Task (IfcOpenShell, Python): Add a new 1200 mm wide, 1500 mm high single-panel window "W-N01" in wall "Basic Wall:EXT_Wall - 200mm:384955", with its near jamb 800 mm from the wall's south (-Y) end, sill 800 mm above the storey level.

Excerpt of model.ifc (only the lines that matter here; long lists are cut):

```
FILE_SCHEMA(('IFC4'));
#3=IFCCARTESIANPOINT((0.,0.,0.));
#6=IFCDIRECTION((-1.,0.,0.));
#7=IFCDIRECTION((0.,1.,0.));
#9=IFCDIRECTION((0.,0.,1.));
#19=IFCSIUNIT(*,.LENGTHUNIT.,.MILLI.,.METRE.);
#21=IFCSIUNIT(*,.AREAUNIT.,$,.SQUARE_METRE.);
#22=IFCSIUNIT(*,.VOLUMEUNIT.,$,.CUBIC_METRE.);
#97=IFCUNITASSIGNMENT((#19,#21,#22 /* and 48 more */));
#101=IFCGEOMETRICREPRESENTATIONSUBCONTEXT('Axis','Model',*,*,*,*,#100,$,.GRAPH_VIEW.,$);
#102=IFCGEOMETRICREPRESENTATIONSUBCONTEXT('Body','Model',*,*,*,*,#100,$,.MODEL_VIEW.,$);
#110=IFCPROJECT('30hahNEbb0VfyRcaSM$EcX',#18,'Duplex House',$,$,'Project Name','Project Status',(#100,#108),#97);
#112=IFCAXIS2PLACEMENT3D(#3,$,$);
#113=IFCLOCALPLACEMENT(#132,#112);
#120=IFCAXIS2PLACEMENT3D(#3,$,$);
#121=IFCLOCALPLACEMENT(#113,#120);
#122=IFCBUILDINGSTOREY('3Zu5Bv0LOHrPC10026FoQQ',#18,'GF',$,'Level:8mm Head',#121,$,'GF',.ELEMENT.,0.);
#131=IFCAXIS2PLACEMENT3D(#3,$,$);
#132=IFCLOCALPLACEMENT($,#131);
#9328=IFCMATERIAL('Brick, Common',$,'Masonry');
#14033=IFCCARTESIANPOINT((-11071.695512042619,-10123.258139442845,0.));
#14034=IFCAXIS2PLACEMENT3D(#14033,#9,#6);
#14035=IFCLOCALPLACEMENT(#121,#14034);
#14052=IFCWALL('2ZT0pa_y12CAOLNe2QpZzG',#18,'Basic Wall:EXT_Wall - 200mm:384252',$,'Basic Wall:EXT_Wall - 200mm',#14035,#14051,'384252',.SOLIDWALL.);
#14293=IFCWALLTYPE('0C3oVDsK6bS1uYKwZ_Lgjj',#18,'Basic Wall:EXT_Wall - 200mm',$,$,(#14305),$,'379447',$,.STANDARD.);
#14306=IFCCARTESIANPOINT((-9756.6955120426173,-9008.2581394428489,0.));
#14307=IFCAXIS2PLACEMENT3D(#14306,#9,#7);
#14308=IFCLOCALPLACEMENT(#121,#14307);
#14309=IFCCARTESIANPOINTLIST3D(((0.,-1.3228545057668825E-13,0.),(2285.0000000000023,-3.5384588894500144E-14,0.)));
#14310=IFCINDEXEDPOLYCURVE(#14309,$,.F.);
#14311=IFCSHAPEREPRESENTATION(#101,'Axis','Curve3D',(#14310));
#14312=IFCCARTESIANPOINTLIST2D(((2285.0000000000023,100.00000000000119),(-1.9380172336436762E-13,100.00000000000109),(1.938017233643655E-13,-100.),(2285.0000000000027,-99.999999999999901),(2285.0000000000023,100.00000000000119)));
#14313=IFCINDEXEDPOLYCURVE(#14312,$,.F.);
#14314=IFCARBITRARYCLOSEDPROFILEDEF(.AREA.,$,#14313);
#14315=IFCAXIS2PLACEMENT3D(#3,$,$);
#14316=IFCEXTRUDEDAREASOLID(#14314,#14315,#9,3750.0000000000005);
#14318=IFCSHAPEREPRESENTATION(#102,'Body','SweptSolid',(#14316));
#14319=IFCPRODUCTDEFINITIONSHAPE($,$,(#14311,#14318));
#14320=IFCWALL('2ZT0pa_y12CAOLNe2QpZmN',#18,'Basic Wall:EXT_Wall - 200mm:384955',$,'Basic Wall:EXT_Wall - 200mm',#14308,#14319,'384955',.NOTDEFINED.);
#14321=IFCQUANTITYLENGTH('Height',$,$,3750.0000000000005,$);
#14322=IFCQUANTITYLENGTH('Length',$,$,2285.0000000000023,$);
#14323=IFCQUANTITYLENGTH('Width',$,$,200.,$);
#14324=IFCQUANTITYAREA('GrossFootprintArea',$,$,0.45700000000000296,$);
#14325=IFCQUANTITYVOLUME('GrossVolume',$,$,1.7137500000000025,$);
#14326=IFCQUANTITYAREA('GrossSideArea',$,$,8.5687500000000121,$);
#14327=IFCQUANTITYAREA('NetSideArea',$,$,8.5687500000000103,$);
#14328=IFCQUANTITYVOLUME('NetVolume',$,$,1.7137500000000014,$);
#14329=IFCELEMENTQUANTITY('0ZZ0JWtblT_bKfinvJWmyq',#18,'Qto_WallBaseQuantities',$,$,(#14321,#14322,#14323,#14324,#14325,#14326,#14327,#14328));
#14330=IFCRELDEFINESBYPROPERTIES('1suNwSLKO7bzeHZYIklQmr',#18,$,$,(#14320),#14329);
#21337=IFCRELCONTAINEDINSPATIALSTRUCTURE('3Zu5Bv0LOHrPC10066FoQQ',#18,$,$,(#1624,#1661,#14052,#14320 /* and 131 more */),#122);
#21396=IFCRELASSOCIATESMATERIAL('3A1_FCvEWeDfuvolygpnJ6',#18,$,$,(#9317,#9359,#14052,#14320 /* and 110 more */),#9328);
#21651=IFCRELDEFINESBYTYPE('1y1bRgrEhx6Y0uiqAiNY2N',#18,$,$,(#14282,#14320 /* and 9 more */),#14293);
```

```python
import numpy as np
import ifcopenshell
import ifcopenshell.api.feature
import ifcopenshell.api.geometry
import ifcopenshell.api.pset
import ifcopenshell.api.root
import ifcopenshell.api.spatial
import ifcopenshell.geom
import ifcopenshell.util.element
import ifcopenshell.util.placement
import ifcopenshell.util.representation
import ifcopenshell.util.shape
import ifcopenshell.util.unit

model = ifcopenshell.open("model.ifc")
unit_scale = ifcopenshell.util.unit.calculate_unit_scale(model)
area_scale = ifcopenshell.util.unit.calculate_unit_scale(model, "AREAUNIT")
volume_scale = ifcopenshell.util.unit.calculate_unit_scale(model, "VOLUMEUNIT")
settings = ifcopenshell.geom.settings()


def volume(element):
    """Net volume in cubic metres, openings subtracted."""
    shape = ifcopenshell.geom.create_shape(settings, element)
    return ifcopenshell.util.shape.get_volume(shape.geometry)


wall = model.by_guid("2ZT0pa_y12CAOLNe2QpZmN")
storey = ifcopenshell.util.element.get_container(wall, ifc_class="IfcBuildingStorey")
context = ifcopenshell.util.representation.get_context(model, "Model", "Body", "MODEL_VIEW")
before = volume(wall)

width, height, from_end, sill = 1.2, 1.5, 0.8, 0.8  # metres

# The wall runs along its own X axis, and the end named is its -X end.
wall_shape = ifcopenshell.geom.create_shape(settings, wall)
x, y, z = ifcopenshell.util.shape.get_vertices(wall_shape.geometry).T
start = x.min() + from_end
face, thickness = float(y.min()), float(y.max() - y.min())
wall_matrix = ifcopenshell.util.placement.get_local_placement(wall.ObjectPlacement)
level = ifcopenshell.util.placement.get_local_placement(storey.ObjectPlacement)[2, 3]


def in_wall(x, y):
    """Placement at x, y metres in the wall's axes, at sill height."""
    matrix = wall_matrix.copy()
    matrix[:, 3] = wall_matrix @ np.array([x / unit_scale, y / unit_scale, 0.0, 1.0])
    matrix[2, 3] = level + sill / unit_scale
    return matrix


# Opening: a box that overshoots both wall faces by 50 mm.
opening = ifcopenshell.api.root.create_entity(model, ifc_class="IfcOpeningElement", predefined_type="OPENING")
box = ifcopenshell.api.geometry.add_wall_representation(
    model, context=context, length=width, height=height, thickness=thickness + 0.1
)
ifcopenshell.api.geometry.assign_representation(model, product=opening, representation=box)
ifcopenshell.api.geometry.edit_object_placement(model, product=opening, matrix=in_wall(start, face - 0.05), is_si=False)
ifcopenshell.api.feature.add_feature(model, feature=opening, element=wall)

window = ifcopenshell.api.root.create_entity(model, ifc_class="IfcWindow", name="W-N01", predefined_type="WINDOW")
window.OverallWidth, window.OverallHeight = width / unit_scale, height / unit_scale
window.PartitioningType = "SINGLE_PANEL"
body = ifcopenshell.api.geometry.add_window_representation(
    model,
    context=context,
    overall_width=window.OverallWidth,
    overall_height=window.OverallHeight,
    partition_type="SINGLE_PANEL",
)
ifcopenshell.api.geometry.assign_representation(model, product=window, representation=body)
ifcopenshell.api.spatial.assign_container(model, products=[window], relating_structure=storey)
ifcopenshell.api.feature.add_filling(model, opening=opening, element=window)

# Centre the window in the wall's thickness.
ifcopenshell.api.geometry.edit_object_placement(model, product=window, matrix=in_wall(start, face), is_si=False)
window_shape = ifcopenshell.geom.create_shape(settings, window)
depth = ifcopenshell.util.shape.get_vertices(window_shape.geometry)[:, 1]
offset = face + thickness / 2 - (depth.min() + depth.max()) / 2
ifcopenshell.api.geometry.edit_object_placement(model, product=window, matrix=in_wall(start, offset), is_si=False)

after = volume(wall)

# Update the wall's stored quantities.
qto = model.by_id(ifcopenshell.util.element.get_pset(wall, "Qto_WallBaseQuantities", should_inherit=False)["id"])
ifcopenshell.api.pset.edit_qto(model, qto=qto, properties={
    "NetSideArea": after / thickness / area_scale,
    "NetVolume": after / volume_scale,
})

print(f"wall volume {before:.3f} -> {after:.3f} m3")

model.write("model_v2.ifc")
```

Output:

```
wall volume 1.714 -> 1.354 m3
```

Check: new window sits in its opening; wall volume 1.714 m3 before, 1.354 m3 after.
